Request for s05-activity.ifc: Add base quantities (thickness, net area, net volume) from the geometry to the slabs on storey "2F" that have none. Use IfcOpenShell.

First a look at what the model holds.

```python
import ifcopenshell
import ifcopenshell.util.element
import ifcopenshell.util.unit

model = ifcopenshell.open("s05-activity.ifc")
print(model.schema)
for unit_type in ("LENGTHUNIT", "AREAUNIT", "VOLUMEUNIT"):
    print(unit_type, ifcopenshell.util.unit.calculate_unit_scale(model, unit_type))
storey = next(s for s in model.by_type("IfcBuildingStorey") if s.Name == "2F")
slabs = [e for e in ifcopenshell.util.element.get_decomposition(storey) if e.is_a("IfcSlab")]
for e in sorted(slabs, key=lambda e: e.id()):
    print(e.id(), e.is_a(), e.Name, list(ifcopenshell.util.element.get_psets(e, qtos_only=True)), sep=" | ")
```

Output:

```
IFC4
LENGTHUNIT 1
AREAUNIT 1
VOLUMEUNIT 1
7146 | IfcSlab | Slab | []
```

```python
import ifcopenshell
import ifcopenshell.api.pset
import ifcopenshell.geom
import ifcopenshell.util.element
import ifcopenshell.util.shape
import ifcopenshell.util.unit

model = ifcopenshell.open("s05-activity.ifc")
unit_scale = ifcopenshell.util.unit.calculate_unit_scale(model)
area_scale = ifcopenshell.util.unit.calculate_unit_scale(model, "AREAUNIT")
volume_scale = ifcopenshell.util.unit.calculate_unit_scale(model, "VOLUMEUNIT")
settings = ifcopenshell.geom.settings()

storey = next(s for s in model.by_type("IfcBuildingStorey") if s.Name == "2F")
slabs = [e for e in ifcopenshell.util.element.get_decomposition(storey) if e.is_a("IfcSlab")]

for e in sorted(slabs, key=lambda e: e.id()):
    if ifcopenshell.util.element.get_psets(e, qtos_only=True, should_inherit=False):
        continue
    # Geometry comes back in metres, in the element's own axes.
    shape = ifcopenshell.geom.create_shape(settings, e)
    values = {
        "Width": ifcopenshell.util.shape.get_z(shape.geometry) / unit_scale,
        "NetArea": ifcopenshell.util.shape.get_footprint_area(shape.geometry) / area_scale,
        "NetVolume": ifcopenshell.util.shape.get_volume(shape.geometry) / volume_scale,
    }
    qto = ifcopenshell.api.pset.add_qto(model, product=e, name="Qto_SlabBaseQuantities")
    ifcopenshell.api.pset.edit_qto(model, qto=qto, properties=values)
    print(e.id(), {k: round(v, 3) for k, v in values.items()})

model.write("s05-activity_updated.ifc")
```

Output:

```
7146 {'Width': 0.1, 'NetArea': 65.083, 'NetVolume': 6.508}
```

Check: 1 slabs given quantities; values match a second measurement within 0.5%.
